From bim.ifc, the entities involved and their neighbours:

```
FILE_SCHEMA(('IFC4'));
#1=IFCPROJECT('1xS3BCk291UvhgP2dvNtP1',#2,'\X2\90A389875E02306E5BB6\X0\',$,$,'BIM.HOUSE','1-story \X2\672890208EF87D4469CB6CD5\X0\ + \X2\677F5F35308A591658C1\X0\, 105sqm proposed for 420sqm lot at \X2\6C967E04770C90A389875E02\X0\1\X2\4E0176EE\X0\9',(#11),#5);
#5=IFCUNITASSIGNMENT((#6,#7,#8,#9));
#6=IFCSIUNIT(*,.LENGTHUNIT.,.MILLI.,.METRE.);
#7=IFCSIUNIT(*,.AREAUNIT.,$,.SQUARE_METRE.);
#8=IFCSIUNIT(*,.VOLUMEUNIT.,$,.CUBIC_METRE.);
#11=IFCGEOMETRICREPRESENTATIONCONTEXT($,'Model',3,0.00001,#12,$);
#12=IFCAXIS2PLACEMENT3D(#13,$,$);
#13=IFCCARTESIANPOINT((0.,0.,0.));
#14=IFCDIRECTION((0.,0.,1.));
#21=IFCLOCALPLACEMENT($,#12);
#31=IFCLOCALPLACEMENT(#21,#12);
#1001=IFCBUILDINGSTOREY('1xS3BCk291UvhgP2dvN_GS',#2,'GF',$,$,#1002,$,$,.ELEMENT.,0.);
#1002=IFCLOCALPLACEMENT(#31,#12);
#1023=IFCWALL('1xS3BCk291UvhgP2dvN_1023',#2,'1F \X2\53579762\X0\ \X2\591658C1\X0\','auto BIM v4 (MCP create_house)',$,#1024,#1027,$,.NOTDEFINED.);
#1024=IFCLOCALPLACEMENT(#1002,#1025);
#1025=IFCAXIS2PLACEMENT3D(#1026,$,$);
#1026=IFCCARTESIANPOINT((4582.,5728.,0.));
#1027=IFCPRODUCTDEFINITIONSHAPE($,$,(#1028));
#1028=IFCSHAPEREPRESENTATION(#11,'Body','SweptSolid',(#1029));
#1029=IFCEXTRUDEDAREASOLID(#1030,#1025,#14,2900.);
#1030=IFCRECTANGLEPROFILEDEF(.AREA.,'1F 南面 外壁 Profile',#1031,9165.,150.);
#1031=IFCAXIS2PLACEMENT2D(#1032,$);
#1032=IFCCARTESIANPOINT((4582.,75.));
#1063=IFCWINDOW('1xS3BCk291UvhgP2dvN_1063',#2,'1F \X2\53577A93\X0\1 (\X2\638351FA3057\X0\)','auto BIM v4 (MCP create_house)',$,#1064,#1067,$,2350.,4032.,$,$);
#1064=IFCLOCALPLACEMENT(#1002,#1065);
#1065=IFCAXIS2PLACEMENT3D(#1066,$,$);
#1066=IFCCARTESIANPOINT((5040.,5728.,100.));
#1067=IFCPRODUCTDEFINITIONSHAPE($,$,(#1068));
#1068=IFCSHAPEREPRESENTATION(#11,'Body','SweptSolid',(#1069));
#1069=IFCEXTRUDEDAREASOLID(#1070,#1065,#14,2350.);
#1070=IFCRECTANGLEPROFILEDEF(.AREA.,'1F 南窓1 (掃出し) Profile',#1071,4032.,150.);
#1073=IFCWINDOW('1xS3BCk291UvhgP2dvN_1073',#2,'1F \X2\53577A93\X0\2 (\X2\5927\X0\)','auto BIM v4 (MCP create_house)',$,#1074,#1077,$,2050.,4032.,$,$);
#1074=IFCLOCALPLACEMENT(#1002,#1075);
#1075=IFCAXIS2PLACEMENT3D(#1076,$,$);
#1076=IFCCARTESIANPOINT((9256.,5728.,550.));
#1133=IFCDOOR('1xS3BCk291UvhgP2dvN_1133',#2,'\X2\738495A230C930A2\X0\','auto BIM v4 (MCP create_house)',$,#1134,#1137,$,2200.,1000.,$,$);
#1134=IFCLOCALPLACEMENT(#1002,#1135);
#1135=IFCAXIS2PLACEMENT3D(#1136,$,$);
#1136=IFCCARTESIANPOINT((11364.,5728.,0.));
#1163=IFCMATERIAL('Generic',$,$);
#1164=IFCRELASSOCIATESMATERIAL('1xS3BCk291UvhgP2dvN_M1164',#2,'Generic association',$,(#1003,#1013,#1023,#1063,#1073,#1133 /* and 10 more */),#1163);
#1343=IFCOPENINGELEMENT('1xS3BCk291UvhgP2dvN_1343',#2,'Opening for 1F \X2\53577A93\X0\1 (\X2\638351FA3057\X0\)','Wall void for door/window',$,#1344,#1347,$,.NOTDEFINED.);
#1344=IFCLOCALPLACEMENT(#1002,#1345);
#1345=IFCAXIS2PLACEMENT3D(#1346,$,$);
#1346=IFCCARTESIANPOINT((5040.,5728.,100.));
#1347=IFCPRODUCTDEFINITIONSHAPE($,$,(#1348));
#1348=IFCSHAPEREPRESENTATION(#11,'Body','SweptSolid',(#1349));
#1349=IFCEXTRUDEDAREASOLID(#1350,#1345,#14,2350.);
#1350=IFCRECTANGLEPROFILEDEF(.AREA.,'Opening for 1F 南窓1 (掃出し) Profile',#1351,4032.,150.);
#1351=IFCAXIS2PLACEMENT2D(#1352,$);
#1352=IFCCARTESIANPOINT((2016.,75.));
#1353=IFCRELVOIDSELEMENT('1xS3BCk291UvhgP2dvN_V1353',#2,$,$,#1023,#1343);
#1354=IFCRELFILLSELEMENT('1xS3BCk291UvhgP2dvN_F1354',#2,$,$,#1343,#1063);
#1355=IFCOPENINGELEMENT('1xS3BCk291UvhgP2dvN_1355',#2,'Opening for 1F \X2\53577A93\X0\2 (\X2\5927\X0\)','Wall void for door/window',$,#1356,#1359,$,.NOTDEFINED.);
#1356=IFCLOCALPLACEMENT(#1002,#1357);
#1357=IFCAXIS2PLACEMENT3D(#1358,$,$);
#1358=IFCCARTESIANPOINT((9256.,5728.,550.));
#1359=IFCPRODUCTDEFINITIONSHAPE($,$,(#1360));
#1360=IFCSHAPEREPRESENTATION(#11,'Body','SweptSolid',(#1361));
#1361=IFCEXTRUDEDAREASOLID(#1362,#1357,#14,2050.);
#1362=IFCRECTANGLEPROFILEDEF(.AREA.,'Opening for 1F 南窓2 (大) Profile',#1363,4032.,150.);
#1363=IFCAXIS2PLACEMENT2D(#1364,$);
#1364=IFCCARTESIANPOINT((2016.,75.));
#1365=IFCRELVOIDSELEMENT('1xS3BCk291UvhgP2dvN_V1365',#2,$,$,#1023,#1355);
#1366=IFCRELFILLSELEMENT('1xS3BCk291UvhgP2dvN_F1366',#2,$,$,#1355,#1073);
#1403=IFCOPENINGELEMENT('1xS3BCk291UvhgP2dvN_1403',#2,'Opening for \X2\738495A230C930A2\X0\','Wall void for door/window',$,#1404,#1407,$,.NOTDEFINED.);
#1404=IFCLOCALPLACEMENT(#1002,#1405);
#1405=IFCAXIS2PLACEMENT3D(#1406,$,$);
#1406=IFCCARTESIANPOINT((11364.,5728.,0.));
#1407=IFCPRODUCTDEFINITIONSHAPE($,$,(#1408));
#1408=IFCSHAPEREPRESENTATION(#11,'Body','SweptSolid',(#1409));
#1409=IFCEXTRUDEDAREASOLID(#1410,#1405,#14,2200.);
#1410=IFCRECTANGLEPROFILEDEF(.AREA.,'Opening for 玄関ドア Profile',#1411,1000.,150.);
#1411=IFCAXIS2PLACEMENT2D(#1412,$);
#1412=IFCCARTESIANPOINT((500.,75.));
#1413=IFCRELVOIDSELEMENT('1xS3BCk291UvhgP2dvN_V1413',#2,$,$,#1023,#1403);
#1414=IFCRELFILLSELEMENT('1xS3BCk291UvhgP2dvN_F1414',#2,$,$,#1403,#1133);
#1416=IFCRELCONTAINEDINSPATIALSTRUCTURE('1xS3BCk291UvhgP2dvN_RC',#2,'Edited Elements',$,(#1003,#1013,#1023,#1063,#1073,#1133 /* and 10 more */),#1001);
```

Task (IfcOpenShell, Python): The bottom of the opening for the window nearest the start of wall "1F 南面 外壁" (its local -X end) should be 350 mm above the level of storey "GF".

```python
import numpy as np
import ifcopenshell
import ifcopenshell.api.geometry
import ifcopenshell.geom
import ifcopenshell.util.element
import ifcopenshell.util.placement
import ifcopenshell.util.shape
import ifcopenshell.util.unit

model = ifcopenshell.open("bim.ifc")
unit_scale = ifcopenshell.util.unit.calculate_unit_scale(model)

window = model.by_guid("1xS3BCk291UvhgP2dvN_1063")
opening = window.FillsVoids[0].RelatingOpeningElement
storey = ifcopenshell.util.element.get_container(window, ifc_class="IfcBuildingStorey")
level = ifcopenshell.util.placement.get_local_placement(storey.ObjectPlacement)[2, 3]

# The opening's origin need not be at the sill, so measure its lowest point.
shape = ifcopenshell.geom.create_shape(ifcopenshell.geom.settings(), opening)
bottom = ifcopenshell.util.shape.get_shape_bottom_elevation(shape, shape.geometry) / unit_scale
dz = level + 350.0 - bottom

shift = np.array([0.0, 0.0, dz])
# The window is not placed relative to its opening, so move both.
for product in (opening, window):
    matrix = ifcopenshell.util.placement.get_local_placement(product.ObjectPlacement)
    matrix[:3, 3] += shift
    ifcopenshell.api.geometry.edit_object_placement(model, product=product, matrix=matrix, is_si=False)

print(f"moved by {dz * unit_scale:+.3f} m")

model.write("bim_rev.ifc")
```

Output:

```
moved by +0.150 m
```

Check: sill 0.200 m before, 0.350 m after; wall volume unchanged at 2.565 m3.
